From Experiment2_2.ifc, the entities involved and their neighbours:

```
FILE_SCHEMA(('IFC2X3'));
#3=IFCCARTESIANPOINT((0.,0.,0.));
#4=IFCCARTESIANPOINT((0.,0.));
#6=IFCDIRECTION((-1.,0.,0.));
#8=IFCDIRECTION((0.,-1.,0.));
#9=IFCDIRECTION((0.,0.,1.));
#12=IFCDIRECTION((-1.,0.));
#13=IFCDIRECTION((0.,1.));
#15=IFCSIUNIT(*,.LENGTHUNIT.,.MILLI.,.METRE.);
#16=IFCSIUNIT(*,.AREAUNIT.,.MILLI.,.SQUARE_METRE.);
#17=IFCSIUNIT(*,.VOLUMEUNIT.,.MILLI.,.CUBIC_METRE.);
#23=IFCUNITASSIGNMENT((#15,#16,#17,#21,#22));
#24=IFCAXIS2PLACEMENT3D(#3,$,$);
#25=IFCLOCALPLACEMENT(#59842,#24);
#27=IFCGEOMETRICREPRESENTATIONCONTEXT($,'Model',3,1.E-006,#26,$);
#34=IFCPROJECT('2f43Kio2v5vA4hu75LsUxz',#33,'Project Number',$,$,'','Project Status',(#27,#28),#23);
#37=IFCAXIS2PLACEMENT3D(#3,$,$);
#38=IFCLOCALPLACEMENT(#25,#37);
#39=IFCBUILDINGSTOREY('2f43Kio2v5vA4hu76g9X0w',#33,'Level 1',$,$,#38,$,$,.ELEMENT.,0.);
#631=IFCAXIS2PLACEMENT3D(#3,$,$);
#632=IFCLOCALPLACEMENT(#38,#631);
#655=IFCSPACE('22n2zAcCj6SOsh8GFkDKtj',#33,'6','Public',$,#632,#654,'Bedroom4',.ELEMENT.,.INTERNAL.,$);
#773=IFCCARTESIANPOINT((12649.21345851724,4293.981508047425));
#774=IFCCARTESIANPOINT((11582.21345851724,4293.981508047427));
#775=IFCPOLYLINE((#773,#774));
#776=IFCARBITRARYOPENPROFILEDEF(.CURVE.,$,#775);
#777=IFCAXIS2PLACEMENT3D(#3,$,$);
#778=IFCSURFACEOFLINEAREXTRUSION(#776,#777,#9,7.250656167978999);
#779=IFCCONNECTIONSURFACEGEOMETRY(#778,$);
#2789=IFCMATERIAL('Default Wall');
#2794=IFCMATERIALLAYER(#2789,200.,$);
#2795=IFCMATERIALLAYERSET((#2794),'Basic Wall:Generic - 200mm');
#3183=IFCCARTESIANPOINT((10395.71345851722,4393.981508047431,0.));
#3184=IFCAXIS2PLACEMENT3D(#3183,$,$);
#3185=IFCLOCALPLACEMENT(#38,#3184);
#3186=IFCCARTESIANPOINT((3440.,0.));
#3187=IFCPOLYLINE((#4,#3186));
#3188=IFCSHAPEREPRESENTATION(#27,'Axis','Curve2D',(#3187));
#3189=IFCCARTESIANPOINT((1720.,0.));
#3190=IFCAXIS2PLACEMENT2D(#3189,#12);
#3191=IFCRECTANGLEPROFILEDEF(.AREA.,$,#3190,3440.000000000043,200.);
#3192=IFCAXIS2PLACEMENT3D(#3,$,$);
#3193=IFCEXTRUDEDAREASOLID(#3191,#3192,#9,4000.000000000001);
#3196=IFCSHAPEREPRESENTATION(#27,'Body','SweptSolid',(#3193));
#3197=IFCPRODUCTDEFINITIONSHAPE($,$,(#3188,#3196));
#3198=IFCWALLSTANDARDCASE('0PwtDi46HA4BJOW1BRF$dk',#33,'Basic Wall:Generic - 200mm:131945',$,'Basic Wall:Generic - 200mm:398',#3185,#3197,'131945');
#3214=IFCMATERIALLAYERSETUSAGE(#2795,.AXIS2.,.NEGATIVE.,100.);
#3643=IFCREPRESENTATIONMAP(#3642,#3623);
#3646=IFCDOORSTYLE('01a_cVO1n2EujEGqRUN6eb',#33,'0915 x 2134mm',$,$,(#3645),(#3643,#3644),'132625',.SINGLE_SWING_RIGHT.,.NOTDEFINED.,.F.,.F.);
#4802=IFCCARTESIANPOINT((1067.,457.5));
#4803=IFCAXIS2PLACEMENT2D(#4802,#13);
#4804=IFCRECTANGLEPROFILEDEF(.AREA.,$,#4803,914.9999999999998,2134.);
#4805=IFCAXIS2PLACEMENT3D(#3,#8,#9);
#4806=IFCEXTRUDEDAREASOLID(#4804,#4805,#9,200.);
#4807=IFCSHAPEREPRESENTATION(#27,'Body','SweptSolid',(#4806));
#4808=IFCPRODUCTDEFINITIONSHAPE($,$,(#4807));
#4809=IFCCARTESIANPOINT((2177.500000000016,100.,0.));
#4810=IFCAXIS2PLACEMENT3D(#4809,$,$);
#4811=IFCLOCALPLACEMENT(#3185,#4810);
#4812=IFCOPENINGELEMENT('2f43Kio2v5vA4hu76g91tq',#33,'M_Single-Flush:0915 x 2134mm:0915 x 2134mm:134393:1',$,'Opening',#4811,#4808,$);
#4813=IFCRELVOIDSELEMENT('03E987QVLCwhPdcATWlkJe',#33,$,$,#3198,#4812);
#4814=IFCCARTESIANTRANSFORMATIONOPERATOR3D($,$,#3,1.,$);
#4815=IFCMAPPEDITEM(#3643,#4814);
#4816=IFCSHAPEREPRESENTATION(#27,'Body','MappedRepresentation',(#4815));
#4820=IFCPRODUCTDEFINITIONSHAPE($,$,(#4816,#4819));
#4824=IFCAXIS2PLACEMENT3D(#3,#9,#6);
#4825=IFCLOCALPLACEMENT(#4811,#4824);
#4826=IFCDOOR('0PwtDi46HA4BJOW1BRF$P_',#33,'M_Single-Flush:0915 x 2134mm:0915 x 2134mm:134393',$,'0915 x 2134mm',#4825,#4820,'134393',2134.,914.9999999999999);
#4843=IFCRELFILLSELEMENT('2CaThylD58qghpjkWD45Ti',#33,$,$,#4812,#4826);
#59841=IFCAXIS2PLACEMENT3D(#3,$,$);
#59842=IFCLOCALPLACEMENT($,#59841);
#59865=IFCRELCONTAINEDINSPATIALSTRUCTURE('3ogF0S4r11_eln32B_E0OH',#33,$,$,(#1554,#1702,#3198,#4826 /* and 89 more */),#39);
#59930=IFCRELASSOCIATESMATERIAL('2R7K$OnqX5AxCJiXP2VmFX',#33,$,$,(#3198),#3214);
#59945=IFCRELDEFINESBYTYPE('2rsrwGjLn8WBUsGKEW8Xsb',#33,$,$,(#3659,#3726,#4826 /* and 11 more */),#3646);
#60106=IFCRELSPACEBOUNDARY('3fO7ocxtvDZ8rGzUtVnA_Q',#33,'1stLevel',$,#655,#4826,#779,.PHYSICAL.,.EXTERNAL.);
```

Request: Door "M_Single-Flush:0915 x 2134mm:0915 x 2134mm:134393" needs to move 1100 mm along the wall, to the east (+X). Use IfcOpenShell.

```python
import numpy as np
import ifcopenshell
import ifcopenshell.api.geometry
import ifcopenshell.util.placement

model = ifcopenshell.open("Experiment2_2.ifc")

door = model.by_guid("0PwtDi46HA4BJOW1BRF$P_")
opening = door.FillsVoids[0].RelatingOpeningElement
wall = opening.VoidsElements[0].RelatingBuildingElement

wall_matrix = ifcopenshell.util.placement.get_local_placement(wall.ObjectPlacement)
shift = wall_matrix[:3, 0] * 1100.0
before = ifcopenshell.util.placement.get_local_placement(door.ObjectPlacement)[:3, 3].copy()

# The door is placed relative to its opening, so it follows when the opening moves.
matrix = ifcopenshell.util.placement.get_local_placement(opening.ObjectPlacement)
matrix[:3, 3] += shift
ifcopenshell.api.geometry.edit_object_placement(
    model, product=opening, matrix=matrix, is_si=False, should_transform_children=True
)

# Space boundary surfaces are stored in each space's coordinates; move them too.
for rel in door.ProvidesBoundaries:
    if not rel.ConnectionGeometry:
        continue
    surface = rel.ConnectionGeometry.SurfaceOnRelatingElement
    space_matrix = ifcopenshell.util.placement.get_local_placement(rel.RelatingSpace.ObjectPlacement)
    point = np.array(surface.Position.Location.Coordinates) + space_matrix[:3, :3].T @ shift
    surface.Position = model.createIfcAxis2Placement3D(
        model.createIfcCartesianPoint(point.tolist()), surface.Position.Axis, surface.Position.RefDirection
    )

after = ifcopenshell.util.placement.get_local_placement(door.ObjectPlacement)[:3, 3]
print("door moved by", (after - before).round(3) + 0.0)

model.write("Experiment2_2_updated.ifc")
```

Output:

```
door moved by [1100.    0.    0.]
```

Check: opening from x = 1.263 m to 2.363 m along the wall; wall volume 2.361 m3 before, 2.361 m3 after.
